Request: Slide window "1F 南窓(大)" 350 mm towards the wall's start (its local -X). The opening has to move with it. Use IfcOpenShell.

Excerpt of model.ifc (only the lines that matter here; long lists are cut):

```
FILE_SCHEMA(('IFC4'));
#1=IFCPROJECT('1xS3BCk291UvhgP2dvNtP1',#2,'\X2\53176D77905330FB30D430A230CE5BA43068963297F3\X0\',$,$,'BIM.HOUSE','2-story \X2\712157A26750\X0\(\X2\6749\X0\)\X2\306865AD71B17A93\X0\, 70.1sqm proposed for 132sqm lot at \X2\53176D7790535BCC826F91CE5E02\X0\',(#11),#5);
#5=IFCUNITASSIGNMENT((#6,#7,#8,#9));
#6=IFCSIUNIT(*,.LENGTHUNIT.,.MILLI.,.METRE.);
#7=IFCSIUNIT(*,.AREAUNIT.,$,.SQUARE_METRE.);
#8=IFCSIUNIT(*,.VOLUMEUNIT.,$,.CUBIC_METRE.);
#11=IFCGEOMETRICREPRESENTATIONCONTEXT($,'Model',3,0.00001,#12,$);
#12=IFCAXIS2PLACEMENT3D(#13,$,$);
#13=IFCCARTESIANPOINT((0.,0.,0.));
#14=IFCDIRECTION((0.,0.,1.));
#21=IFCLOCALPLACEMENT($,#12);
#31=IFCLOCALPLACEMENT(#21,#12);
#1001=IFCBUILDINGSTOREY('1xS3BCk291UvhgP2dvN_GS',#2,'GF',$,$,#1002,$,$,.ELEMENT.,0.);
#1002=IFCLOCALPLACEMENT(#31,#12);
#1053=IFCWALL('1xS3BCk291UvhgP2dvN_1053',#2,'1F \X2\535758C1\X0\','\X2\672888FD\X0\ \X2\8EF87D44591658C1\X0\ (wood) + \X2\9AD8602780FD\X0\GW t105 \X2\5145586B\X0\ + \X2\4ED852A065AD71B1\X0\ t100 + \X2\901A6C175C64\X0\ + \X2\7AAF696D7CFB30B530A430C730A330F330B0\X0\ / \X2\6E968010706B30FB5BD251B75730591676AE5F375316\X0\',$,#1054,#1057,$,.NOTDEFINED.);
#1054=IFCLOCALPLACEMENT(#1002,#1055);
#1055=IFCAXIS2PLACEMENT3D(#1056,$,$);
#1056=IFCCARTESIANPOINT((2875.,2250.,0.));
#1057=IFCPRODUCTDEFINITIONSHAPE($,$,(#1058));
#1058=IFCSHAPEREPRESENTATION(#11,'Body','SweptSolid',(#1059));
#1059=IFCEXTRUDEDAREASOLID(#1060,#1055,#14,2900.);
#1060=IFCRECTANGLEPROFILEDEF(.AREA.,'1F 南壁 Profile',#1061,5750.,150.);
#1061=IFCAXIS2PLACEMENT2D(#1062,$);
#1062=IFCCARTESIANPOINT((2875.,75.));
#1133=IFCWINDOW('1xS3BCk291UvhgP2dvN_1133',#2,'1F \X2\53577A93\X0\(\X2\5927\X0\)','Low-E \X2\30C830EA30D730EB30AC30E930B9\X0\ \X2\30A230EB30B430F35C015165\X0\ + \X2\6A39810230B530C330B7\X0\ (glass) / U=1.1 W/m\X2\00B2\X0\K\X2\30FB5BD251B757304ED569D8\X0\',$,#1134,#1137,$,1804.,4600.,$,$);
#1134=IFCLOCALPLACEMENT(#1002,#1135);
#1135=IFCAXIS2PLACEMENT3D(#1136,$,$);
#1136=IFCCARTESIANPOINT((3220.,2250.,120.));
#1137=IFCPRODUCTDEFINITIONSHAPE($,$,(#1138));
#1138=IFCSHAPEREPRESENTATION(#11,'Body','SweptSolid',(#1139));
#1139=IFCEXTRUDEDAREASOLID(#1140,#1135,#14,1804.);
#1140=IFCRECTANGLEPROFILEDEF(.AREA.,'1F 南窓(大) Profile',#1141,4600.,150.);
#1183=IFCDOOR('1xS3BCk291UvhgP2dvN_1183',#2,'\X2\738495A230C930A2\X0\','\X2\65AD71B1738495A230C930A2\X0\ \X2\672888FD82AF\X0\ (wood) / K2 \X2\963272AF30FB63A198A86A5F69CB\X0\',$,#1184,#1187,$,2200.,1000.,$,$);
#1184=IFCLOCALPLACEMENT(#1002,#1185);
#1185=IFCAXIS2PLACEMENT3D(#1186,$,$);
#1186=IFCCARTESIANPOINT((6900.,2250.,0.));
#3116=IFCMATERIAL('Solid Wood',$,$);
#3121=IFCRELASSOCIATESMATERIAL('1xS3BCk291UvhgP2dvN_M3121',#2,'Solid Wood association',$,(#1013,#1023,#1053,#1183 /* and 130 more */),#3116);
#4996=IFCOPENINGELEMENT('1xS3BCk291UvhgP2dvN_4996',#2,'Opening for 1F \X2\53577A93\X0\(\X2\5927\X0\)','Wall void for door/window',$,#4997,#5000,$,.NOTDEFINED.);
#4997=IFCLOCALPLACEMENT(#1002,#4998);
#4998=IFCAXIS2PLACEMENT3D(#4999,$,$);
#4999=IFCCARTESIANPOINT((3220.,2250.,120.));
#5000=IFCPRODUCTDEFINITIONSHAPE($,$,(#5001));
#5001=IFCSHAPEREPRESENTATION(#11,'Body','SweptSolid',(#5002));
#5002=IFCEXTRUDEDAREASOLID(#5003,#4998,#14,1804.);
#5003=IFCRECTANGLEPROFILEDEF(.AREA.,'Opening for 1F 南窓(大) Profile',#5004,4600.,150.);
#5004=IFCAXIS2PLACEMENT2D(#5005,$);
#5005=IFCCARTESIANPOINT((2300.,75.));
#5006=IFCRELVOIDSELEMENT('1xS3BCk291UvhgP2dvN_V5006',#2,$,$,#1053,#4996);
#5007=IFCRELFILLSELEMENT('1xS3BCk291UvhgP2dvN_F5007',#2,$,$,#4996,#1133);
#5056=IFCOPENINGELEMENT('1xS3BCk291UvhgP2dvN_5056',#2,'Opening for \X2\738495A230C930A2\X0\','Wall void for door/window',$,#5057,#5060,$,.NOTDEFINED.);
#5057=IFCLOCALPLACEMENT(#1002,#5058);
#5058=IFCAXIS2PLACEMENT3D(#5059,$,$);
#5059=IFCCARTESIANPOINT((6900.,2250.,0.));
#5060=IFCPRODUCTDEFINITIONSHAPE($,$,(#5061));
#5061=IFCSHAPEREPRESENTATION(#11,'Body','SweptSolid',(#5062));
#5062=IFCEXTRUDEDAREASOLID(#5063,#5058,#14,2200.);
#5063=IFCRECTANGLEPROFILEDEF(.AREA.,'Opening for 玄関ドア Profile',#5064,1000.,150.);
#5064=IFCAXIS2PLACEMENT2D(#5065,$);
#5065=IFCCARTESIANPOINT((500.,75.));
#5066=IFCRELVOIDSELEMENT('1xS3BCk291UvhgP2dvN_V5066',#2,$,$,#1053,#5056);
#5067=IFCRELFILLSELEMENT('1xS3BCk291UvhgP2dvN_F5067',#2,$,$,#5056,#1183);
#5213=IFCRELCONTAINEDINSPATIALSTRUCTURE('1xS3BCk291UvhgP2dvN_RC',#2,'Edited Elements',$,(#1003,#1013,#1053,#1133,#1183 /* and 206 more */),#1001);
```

```python
import ifcopenshell
import ifcopenshell.api.geometry
import ifcopenshell.util.placement

model = ifcopenshell.open("model.ifc")

window = model.by_id(1133)
opening = window.FillsVoids[0].RelatingOpeningElement
wall = opening.VoidsElements[0].RelatingBuildingElement

wall_matrix = ifcopenshell.util.placement.get_local_placement(wall.ObjectPlacement)
shift = wall_matrix[:3, 0] * -350.0
before = ifcopenshell.util.placement.get_local_placement(window.ObjectPlacement)[:3, 3].copy()

# The window is not placed relative to its opening, so move both.
for product in (opening, window):
    matrix = ifcopenshell.util.placement.get_local_placement(product.ObjectPlacement)
    matrix[:3, 3] += shift
    ifcopenshell.api.geometry.edit_object_placement(model, product=product, matrix=matrix, is_si=False)

after = ifcopenshell.util.placement.get_local_placement(window.ObjectPlacement)[:3, 3]
print("window moved by", (after - before).round(3) + 0.0)

model.write("model_edited.ifc")
```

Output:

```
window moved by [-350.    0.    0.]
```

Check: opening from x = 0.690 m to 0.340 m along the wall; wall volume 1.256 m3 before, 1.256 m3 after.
